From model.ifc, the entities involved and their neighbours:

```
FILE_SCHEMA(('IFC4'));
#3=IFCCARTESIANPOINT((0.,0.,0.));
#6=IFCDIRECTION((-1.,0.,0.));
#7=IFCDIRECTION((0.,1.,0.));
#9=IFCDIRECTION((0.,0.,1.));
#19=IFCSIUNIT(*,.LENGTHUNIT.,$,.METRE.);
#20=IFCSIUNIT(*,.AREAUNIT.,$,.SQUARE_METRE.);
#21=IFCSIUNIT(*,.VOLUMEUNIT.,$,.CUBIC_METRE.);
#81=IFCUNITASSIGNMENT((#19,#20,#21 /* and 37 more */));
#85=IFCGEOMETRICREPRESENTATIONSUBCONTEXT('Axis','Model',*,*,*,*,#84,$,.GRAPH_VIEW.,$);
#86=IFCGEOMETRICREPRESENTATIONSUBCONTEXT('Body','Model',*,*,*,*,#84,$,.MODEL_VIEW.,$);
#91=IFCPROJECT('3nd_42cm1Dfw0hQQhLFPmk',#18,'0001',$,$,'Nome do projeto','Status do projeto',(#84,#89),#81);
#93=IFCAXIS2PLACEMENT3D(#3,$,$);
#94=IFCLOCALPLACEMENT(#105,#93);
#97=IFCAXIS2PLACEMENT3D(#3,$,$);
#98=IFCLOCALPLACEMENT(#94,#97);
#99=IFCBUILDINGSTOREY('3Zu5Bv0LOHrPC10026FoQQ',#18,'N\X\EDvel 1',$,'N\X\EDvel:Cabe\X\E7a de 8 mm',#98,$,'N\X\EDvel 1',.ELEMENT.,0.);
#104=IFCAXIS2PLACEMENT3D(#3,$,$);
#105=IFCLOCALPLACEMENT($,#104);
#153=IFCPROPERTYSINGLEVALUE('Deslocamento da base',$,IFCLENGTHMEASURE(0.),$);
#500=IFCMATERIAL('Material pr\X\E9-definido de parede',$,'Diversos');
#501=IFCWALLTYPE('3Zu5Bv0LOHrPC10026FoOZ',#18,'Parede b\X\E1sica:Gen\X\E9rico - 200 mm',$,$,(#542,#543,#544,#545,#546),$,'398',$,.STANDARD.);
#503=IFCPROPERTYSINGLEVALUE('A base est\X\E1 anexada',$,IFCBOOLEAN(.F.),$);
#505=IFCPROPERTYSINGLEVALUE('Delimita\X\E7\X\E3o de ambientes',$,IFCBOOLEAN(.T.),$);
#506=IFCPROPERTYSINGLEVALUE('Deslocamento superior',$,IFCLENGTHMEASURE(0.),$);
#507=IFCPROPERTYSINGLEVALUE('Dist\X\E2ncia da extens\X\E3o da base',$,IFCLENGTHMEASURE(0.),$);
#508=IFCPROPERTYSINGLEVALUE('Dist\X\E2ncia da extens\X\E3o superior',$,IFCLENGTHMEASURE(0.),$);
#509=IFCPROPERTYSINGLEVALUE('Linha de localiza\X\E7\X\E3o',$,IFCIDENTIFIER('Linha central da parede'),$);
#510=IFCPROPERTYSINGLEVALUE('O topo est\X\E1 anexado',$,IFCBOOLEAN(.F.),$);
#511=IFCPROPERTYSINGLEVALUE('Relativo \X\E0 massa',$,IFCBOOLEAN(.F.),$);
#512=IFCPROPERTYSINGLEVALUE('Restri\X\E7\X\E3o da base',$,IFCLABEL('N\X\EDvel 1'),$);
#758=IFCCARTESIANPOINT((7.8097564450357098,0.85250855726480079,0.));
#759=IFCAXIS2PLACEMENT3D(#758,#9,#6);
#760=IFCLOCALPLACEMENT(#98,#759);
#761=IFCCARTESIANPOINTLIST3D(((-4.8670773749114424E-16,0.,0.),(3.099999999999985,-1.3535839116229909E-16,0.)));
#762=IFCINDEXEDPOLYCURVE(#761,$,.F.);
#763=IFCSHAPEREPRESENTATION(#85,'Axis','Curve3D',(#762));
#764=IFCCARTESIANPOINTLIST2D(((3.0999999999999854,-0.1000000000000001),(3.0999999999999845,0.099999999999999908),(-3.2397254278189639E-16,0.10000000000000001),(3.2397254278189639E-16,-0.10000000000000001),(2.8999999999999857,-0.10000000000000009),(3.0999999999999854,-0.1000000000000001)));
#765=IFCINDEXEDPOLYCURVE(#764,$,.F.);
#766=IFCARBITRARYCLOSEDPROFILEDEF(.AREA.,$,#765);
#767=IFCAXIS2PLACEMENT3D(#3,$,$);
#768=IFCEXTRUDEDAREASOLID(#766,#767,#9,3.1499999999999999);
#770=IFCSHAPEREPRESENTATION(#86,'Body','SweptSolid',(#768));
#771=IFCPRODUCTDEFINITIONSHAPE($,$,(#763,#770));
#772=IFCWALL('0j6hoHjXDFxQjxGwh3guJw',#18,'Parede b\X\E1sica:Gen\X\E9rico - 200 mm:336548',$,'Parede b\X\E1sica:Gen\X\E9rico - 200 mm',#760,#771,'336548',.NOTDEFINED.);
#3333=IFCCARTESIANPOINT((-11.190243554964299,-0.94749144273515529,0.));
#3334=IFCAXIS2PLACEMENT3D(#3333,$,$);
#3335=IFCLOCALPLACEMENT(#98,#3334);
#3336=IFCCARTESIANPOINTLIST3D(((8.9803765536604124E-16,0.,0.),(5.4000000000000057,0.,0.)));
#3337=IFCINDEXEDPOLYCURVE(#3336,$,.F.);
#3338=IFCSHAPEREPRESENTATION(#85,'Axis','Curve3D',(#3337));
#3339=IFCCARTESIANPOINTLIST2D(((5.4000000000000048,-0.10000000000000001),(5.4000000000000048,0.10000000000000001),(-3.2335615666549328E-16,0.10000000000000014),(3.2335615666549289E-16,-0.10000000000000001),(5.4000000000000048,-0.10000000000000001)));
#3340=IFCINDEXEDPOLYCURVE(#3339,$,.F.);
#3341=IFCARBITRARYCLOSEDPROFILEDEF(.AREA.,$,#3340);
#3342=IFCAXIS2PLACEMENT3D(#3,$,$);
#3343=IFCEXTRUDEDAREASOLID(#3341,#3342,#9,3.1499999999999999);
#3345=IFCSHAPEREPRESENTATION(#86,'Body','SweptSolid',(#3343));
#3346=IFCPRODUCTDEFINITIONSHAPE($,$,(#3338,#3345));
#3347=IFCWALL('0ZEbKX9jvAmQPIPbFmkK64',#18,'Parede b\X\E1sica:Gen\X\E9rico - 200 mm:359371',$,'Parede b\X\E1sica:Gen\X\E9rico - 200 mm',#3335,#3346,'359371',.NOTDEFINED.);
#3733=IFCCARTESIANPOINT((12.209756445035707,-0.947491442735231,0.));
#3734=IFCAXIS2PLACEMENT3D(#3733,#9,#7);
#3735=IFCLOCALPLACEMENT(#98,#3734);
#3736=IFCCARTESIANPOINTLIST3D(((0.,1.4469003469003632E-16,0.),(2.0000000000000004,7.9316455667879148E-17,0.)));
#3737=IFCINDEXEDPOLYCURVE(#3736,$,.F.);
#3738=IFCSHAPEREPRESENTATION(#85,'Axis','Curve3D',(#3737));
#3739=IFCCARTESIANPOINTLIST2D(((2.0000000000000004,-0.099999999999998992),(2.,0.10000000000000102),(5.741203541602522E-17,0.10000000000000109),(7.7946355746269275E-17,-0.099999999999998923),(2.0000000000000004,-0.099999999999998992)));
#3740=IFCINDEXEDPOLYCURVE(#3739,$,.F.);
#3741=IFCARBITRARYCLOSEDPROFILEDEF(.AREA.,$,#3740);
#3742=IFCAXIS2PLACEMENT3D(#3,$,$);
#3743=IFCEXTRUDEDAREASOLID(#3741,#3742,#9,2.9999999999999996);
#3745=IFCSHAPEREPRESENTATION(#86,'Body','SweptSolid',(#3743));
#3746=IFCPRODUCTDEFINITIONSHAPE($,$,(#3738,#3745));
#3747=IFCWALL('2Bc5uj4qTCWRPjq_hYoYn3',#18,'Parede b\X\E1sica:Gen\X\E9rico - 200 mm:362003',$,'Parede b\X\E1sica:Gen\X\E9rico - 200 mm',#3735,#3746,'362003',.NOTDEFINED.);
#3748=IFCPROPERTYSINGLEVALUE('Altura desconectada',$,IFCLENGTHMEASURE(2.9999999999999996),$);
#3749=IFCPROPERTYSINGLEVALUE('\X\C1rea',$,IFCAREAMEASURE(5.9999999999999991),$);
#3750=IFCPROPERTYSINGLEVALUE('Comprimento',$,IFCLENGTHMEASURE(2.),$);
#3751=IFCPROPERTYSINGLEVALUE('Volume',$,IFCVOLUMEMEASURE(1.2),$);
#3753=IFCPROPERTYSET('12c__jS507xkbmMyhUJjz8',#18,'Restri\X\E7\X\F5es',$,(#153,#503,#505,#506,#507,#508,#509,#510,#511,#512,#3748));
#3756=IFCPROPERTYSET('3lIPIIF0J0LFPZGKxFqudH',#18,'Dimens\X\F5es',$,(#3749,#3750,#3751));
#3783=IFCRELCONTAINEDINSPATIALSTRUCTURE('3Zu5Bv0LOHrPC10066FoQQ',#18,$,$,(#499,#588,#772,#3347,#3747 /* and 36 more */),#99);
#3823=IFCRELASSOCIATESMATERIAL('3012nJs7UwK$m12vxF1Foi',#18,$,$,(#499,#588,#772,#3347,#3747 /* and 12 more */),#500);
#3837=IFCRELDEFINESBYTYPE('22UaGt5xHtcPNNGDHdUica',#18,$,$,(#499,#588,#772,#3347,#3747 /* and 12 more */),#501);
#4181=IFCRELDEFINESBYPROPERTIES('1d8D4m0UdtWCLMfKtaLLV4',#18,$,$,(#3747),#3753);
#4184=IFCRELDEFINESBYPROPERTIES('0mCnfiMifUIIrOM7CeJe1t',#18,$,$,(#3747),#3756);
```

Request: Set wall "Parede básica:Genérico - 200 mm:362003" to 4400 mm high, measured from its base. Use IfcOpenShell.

```python
import ifcopenshell
import ifcopenshell.api.pset
import ifcopenshell.geom
import ifcopenshell.util.element
import ifcopenshell.util.representation
import ifcopenshell.util.shape
import ifcopenshell.util.unit

model = ifcopenshell.open("model.ifc")
area_scale = ifcopenshell.util.unit.calculate_unit_scale(model, "AREAUNIT")
volume_scale = ifcopenshell.util.unit.calculate_unit_scale(model, "VOLUMEUNIT")
settings = ifcopenshell.geom.settings()


def volume(element):
    """Net volume in cubic metres, openings subtracted."""
    shape = ifcopenshell.geom.create_shape(settings, element)
    return ifcopenshell.util.shape.get_volume(shape.geometry)


wall = model.by_guid("2Bc5uj4qTCWRPjq_hYoYn3")
before = volume(wall)

body = ifcopenshell.util.representation.get_representation(wall, "Model", "Body")
solid = body.Items[0]
old_height = solid.Depth
solid.Depth = 4.4
after = volume(wall)
thickness = 0.2  # wall thickness in metres

# Update the stored height, areas and volumes.
pset = model.by_id(ifcopenshell.util.element.get_pset(wall, "Restrições", should_inherit=False)["id"])
ifcopenshell.api.pset.edit_pset(model, pset=pset, properties={
    "Altura desconectada": model.create_entity("IfcLengthMeasure", solid.Depth),
})
pset = model.by_id(ifcopenshell.util.element.get_pset(wall, "Dimensões", should_inherit=False)["id"])
ifcopenshell.api.pset.edit_pset(model, pset=pset, properties={
    "Área": model.create_entity("IfcAreaMeasure", after / thickness / area_scale),
    "Volume": model.create_entity("IfcVolumeMeasure", after / volume_scale),
})

print(f"height {old_height:g} -> {solid.Depth:g}, volume {before:.3f} -> {after:.3f} m3")

model.write("model_v2.ifc")
```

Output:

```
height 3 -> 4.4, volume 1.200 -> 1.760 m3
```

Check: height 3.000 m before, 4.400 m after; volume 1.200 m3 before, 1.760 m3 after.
